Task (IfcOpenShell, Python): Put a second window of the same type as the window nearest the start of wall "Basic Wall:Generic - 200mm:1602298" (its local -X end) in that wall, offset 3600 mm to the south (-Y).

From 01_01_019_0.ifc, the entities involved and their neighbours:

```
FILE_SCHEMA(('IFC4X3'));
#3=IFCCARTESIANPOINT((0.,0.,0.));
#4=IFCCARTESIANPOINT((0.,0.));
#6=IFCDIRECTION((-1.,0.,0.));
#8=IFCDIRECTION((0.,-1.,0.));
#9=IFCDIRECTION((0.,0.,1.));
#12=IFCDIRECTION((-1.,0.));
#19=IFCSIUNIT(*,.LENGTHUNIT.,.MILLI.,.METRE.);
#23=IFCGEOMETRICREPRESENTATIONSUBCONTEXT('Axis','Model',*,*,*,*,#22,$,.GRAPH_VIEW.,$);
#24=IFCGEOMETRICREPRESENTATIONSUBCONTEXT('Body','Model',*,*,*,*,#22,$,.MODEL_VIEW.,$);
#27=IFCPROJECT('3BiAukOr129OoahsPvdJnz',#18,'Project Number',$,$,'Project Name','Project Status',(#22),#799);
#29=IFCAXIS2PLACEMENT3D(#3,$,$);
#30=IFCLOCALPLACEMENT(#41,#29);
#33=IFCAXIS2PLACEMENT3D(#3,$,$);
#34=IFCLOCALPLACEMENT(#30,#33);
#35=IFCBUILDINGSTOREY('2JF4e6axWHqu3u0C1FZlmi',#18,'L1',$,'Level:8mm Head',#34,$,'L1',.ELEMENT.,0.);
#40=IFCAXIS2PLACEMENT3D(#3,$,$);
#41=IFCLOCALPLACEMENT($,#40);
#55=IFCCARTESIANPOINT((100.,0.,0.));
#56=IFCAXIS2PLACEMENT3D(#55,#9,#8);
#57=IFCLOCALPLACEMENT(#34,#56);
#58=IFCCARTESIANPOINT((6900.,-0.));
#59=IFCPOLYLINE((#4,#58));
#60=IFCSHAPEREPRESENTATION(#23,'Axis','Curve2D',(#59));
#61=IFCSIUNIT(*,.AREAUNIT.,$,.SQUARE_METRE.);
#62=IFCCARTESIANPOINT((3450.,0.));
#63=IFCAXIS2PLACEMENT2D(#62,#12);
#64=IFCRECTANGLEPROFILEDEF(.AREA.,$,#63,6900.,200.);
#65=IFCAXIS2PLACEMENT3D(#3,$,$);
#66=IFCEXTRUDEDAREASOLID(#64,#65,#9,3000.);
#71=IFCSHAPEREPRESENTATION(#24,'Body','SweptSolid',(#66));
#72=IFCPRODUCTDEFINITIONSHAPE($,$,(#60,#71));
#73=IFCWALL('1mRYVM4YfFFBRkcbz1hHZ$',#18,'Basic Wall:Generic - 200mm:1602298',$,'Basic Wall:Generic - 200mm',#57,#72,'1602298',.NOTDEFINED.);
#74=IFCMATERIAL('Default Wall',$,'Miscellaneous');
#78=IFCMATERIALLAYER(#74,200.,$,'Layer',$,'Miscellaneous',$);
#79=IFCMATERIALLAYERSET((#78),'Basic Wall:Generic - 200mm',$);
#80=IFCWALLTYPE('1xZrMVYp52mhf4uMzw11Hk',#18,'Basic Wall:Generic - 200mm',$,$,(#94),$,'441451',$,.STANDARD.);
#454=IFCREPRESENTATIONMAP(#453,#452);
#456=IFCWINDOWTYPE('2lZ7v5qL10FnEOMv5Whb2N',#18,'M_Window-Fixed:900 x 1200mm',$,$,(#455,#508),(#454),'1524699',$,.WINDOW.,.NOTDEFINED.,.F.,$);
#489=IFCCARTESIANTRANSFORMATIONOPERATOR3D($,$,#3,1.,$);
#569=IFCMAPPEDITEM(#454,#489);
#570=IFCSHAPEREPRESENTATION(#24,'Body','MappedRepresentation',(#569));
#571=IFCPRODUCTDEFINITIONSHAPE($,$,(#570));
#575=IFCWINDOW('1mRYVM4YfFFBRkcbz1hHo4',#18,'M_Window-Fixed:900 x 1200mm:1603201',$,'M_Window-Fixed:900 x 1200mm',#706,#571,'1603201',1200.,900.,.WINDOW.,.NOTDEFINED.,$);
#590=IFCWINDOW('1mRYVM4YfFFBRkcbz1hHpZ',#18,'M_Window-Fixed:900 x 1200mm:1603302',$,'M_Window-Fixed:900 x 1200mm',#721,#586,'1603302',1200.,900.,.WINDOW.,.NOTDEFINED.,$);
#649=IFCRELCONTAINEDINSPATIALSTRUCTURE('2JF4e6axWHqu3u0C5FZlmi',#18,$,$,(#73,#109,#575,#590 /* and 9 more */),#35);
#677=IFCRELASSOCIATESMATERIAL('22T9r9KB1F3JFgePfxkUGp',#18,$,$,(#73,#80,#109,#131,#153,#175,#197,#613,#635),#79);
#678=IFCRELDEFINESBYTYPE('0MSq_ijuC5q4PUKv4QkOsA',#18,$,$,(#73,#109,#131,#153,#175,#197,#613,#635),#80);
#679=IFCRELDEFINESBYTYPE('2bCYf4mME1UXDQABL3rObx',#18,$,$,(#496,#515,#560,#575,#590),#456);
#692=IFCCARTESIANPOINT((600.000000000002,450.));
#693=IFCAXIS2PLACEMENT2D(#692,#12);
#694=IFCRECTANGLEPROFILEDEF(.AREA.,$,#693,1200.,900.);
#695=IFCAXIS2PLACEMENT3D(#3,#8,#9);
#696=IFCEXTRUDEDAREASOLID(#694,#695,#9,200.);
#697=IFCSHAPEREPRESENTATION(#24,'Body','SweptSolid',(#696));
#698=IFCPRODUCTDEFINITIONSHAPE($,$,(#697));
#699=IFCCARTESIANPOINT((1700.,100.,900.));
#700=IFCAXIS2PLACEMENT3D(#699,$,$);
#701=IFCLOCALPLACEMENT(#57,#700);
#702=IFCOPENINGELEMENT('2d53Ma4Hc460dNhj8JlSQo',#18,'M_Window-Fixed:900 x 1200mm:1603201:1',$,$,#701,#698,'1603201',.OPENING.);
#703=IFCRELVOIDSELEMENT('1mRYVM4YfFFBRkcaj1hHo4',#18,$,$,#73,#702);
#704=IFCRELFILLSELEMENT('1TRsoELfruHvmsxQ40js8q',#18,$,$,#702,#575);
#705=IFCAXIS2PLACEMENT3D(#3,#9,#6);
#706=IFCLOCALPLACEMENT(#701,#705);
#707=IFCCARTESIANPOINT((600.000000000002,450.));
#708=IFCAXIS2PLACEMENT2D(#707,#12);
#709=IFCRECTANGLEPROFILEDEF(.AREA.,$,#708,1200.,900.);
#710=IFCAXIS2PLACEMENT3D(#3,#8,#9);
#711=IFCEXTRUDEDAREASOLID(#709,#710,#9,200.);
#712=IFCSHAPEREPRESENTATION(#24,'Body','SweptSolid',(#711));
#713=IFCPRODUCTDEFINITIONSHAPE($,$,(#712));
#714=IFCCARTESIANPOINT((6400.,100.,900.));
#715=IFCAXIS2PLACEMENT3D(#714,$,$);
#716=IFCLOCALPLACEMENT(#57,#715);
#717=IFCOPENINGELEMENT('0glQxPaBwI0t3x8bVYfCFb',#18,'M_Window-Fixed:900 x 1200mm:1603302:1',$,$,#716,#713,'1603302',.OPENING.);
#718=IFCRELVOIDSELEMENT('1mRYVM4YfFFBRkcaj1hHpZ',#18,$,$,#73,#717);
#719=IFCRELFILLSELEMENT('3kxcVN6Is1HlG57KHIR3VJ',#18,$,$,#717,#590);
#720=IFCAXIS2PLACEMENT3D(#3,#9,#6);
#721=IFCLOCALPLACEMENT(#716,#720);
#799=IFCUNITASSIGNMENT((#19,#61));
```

```python
import ifcopenshell
import ifcopenshell.api.feature
import ifcopenshell.api.geometry
import ifcopenshell.api.root
import ifcopenshell.geom
import ifcopenshell.util.element
import ifcopenshell.util.placement
import ifcopenshell.util.shape
import ifcopenshell.util.unit

model = ifcopenshell.open("01_01_019_0.ifc")
unit_scale = ifcopenshell.util.unit.calculate_unit_scale(model)
settings = ifcopenshell.geom.settings()


def volume(element):
    """Net volume in cubic metres, openings subtracted."""
    shape = ifcopenshell.geom.create_shape(settings, element)
    return ifcopenshell.util.shape.get_volume(shape.geometry)


def reuse_history(source, copy):
    """copy_class also copies each property set's owner history, people and application; keep the originals."""
    for rel in copy.IsDefinedBy:
        if rel.is_a("IfcRelDefinesByProperties") and (history := rel.RelatingPropertyDefinition.OwnerHistory):
            rel.RelatingPropertyDefinition.OwnerHistory = source.OwnerHistory
            ifcopenshell.util.element.remove_deep2(model, history)


window = model.by_id(575)
opening = window.FillsVoids[0].RelatingOpeningElement
wall = opening.VoidsElements[0].RelatingBuildingElement
before = volume(wall)
shift = ifcopenshell.util.placement.get_local_placement(wall.ObjectPlacement)[:3, 0] * 3.6 / unit_scale

# copy_class copies the void relationship, type, container and properties, but no geometry.
new_opening = ifcopenshell.api.root.copy_class(model, product=opening)
new_opening.Representation = ifcopenshell.util.element.copy_deep(
    model, opening.Representation, exclude=["IfcGeometricRepresentationContext", "IfcRepresentationMap"]
)
new_opening.Name = "M_Window-Fixed:900 x 1200mm"
new_opening.Tag = None
new_window = ifcopenshell.api.root.copy_class(model, product=window)
new_window.Representation = ifcopenshell.util.element.copy_deep(
    model, window.Representation, exclude=["IfcGeometricRepresentationContext", "IfcRepresentationMap"]
)
new_window.Name = "M_Window-Fixed:900 x 1200mm"
new_window.Tag = None
reuse_history(window, new_window)
ifcopenshell.api.feature.add_filling(model, opening=new_opening, element=new_window)

for old, new in ((opening, new_opening), (window, new_window)):
    matrix = ifcopenshell.util.placement.get_local_placement(old.ObjectPlacement)
    matrix[:3, 3] += shift
    ifcopenshell.api.geometry.edit_object_placement(model, product=new, matrix=matrix, is_si=False)

after = volume(wall)

print(f"wall volume {before:.3f} -> {after:.3f} m3")

model.write("01_01_019_0_rev.ifc")
```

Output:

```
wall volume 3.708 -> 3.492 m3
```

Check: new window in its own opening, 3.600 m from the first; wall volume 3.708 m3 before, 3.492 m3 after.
